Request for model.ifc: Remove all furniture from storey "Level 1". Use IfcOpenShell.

First a look at what the model holds.

```python
import ifcopenshell
import ifcopenshell.util.element

model = ifcopenshell.open("model.ifc")
print(model.schema)
storey = next(s for s in model.by_type("IfcBuildingStorey") if s.Name == "Level 1")
furniture = [e for e in ifcopenshell.util.element.get_decomposition(storey) if e.is_a("IfcFurnishingElement")]
seen = {}
for e in furniture:
    element_type = ifcopenshell.util.element.get_type(e)
    name = element_type.Name if element_type not in (None, e) else None
    seen[name] = seen.get(name, 0) + 1
for name, count in sorted(seen.items(), key=str):
    print(count, "x", name)
```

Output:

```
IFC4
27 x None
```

```python
import ifcopenshell
import ifcopenshell.api.root
import ifcopenshell.util.element

model = ifcopenshell.open("model.ifc")

storey = next(s for s in model.by_type("IfcBuildingStorey") if s.Name == "Level 1")
furniture = [e for e in ifcopenshell.util.element.get_decomposition(storey) if e.is_a("IfcFurnishingElement")]

for e in furniture:
    ifcopenshell.api.root.remove_product(model, product=e)
print(len(furniture), "removed")

model.write("model_edited.ifc")
```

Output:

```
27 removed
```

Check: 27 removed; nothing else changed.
